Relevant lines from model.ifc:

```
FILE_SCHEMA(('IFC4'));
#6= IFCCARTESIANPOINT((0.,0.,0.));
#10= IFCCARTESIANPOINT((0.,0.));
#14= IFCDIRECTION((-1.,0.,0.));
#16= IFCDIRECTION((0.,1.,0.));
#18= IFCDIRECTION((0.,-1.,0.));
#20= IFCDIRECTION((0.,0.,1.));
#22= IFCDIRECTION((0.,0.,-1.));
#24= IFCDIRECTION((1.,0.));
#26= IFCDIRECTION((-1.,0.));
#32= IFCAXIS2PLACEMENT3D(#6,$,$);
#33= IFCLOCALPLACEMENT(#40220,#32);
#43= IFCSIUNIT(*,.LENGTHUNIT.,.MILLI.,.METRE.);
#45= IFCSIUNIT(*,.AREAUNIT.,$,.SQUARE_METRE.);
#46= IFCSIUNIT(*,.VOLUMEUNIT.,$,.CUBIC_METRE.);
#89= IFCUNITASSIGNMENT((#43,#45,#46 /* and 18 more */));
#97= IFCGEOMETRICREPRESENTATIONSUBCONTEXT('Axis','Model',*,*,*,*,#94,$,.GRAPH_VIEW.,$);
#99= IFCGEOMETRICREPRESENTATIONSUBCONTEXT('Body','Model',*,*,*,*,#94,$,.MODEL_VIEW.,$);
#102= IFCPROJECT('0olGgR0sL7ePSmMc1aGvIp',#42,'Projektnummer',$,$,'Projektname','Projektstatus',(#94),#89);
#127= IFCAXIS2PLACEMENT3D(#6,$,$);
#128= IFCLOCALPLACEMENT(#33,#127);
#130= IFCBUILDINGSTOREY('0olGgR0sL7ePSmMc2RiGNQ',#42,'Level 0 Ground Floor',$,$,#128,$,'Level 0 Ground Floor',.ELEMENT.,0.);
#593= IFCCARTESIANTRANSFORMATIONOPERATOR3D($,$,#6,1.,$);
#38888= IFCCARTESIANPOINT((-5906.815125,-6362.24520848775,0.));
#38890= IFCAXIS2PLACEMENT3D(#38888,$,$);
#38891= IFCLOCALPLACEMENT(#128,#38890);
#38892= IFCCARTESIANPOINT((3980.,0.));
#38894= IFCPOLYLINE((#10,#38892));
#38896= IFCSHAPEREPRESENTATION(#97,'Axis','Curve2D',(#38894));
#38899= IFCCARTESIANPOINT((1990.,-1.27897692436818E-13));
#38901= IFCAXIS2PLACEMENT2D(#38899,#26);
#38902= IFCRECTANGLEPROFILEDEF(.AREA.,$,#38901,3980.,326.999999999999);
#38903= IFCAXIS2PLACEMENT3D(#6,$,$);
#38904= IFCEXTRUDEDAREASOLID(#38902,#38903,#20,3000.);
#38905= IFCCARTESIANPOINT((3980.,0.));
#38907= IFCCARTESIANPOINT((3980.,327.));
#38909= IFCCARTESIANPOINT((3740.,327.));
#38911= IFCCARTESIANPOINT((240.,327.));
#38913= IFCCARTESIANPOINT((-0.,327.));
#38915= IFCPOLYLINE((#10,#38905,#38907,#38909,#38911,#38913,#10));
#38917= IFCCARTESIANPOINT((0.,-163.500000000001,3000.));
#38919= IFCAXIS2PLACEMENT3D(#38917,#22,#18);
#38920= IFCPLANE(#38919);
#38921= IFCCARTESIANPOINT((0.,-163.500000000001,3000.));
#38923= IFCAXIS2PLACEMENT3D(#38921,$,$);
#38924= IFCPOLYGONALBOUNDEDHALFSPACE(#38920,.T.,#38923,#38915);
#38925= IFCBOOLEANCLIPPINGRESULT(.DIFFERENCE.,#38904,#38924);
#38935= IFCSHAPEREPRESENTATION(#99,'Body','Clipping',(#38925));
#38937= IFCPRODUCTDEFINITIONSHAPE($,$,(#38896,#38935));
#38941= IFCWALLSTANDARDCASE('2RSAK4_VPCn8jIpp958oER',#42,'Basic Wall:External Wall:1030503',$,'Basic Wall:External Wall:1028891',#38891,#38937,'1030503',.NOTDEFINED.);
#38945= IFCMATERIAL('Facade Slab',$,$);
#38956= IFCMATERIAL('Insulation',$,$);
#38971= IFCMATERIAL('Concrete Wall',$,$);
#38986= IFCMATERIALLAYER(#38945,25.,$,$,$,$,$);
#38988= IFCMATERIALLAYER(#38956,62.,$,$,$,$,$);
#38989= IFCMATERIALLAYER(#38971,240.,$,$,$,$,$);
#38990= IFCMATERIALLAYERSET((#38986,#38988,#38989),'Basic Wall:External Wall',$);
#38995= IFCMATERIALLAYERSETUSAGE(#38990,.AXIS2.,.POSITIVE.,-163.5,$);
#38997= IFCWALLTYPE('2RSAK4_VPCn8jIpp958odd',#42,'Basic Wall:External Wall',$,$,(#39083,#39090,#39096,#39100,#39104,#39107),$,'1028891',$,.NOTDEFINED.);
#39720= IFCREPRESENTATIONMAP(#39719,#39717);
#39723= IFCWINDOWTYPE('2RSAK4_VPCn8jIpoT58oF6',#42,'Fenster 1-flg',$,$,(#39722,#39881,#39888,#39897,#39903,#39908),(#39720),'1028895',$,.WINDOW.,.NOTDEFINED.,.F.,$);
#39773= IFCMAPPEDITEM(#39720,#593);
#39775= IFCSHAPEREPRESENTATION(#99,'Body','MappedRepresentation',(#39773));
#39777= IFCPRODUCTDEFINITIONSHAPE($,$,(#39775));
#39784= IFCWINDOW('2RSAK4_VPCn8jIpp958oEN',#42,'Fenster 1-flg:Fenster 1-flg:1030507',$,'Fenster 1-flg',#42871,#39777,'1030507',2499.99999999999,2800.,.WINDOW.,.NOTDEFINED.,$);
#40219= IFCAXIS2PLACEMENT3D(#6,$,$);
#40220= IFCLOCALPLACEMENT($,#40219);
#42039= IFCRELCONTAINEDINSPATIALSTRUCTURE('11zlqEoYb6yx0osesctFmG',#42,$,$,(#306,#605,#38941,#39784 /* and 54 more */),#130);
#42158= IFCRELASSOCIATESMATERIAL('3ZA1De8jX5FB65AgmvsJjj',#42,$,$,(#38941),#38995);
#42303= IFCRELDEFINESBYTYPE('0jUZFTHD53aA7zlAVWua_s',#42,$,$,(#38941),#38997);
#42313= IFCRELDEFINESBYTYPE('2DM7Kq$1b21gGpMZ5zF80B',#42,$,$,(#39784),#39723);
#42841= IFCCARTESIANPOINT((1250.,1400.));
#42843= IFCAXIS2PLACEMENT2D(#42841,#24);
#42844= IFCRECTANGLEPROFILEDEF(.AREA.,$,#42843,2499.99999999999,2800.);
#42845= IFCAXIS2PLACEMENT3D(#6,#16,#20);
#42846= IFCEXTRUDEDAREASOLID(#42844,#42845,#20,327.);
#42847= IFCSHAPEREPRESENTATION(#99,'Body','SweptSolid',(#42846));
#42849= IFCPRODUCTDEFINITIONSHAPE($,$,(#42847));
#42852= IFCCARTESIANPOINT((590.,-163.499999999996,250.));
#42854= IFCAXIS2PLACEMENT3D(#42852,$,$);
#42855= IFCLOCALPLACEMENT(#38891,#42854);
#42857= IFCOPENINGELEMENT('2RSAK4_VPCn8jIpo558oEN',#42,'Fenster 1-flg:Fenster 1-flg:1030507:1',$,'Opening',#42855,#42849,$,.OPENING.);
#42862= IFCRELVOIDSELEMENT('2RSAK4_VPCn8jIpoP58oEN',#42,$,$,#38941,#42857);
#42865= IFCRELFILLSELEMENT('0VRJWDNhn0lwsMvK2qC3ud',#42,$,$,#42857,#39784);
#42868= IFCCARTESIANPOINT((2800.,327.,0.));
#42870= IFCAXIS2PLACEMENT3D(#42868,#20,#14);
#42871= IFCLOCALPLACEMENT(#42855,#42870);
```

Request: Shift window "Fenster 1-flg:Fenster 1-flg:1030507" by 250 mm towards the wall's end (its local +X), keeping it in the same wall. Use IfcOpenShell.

```python
import ifcopenshell
import ifcopenshell.api.geometry
import ifcopenshell.util.placement
import ifcopenshell.util.unit

model = ifcopenshell.open("model.ifc")
unit_scale = ifcopenshell.util.unit.calculate_unit_scale(model)

window = model.by_guid("2RSAK4_VPCn8jIpp958oEN")
opening = window.FillsVoids[0].RelatingOpeningElement
wall = opening.VoidsElements[0].RelatingBuildingElement

wall_matrix = ifcopenshell.util.placement.get_local_placement(wall.ObjectPlacement)
shift = wall_matrix[:3, 0] * 0.25 / unit_scale
before = ifcopenshell.util.placement.get_local_placement(window.ObjectPlacement)[:3, 3].copy()

# The window is placed relative to its opening, so it follows when the opening moves.
matrix = ifcopenshell.util.placement.get_local_placement(opening.ObjectPlacement)
matrix[:3, 3] += shift
ifcopenshell.api.geometry.edit_object_placement(
    model, product=opening, matrix=matrix, is_si=False, should_transform_children=True
)

after = ifcopenshell.util.placement.get_local_placement(window.ObjectPlacement)[:3, 3]
print("window moved by", (after - before).round(3) + 0.0)

model.write("model_updated.ifc")
```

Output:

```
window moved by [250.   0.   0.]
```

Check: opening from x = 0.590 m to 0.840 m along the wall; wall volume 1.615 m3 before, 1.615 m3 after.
